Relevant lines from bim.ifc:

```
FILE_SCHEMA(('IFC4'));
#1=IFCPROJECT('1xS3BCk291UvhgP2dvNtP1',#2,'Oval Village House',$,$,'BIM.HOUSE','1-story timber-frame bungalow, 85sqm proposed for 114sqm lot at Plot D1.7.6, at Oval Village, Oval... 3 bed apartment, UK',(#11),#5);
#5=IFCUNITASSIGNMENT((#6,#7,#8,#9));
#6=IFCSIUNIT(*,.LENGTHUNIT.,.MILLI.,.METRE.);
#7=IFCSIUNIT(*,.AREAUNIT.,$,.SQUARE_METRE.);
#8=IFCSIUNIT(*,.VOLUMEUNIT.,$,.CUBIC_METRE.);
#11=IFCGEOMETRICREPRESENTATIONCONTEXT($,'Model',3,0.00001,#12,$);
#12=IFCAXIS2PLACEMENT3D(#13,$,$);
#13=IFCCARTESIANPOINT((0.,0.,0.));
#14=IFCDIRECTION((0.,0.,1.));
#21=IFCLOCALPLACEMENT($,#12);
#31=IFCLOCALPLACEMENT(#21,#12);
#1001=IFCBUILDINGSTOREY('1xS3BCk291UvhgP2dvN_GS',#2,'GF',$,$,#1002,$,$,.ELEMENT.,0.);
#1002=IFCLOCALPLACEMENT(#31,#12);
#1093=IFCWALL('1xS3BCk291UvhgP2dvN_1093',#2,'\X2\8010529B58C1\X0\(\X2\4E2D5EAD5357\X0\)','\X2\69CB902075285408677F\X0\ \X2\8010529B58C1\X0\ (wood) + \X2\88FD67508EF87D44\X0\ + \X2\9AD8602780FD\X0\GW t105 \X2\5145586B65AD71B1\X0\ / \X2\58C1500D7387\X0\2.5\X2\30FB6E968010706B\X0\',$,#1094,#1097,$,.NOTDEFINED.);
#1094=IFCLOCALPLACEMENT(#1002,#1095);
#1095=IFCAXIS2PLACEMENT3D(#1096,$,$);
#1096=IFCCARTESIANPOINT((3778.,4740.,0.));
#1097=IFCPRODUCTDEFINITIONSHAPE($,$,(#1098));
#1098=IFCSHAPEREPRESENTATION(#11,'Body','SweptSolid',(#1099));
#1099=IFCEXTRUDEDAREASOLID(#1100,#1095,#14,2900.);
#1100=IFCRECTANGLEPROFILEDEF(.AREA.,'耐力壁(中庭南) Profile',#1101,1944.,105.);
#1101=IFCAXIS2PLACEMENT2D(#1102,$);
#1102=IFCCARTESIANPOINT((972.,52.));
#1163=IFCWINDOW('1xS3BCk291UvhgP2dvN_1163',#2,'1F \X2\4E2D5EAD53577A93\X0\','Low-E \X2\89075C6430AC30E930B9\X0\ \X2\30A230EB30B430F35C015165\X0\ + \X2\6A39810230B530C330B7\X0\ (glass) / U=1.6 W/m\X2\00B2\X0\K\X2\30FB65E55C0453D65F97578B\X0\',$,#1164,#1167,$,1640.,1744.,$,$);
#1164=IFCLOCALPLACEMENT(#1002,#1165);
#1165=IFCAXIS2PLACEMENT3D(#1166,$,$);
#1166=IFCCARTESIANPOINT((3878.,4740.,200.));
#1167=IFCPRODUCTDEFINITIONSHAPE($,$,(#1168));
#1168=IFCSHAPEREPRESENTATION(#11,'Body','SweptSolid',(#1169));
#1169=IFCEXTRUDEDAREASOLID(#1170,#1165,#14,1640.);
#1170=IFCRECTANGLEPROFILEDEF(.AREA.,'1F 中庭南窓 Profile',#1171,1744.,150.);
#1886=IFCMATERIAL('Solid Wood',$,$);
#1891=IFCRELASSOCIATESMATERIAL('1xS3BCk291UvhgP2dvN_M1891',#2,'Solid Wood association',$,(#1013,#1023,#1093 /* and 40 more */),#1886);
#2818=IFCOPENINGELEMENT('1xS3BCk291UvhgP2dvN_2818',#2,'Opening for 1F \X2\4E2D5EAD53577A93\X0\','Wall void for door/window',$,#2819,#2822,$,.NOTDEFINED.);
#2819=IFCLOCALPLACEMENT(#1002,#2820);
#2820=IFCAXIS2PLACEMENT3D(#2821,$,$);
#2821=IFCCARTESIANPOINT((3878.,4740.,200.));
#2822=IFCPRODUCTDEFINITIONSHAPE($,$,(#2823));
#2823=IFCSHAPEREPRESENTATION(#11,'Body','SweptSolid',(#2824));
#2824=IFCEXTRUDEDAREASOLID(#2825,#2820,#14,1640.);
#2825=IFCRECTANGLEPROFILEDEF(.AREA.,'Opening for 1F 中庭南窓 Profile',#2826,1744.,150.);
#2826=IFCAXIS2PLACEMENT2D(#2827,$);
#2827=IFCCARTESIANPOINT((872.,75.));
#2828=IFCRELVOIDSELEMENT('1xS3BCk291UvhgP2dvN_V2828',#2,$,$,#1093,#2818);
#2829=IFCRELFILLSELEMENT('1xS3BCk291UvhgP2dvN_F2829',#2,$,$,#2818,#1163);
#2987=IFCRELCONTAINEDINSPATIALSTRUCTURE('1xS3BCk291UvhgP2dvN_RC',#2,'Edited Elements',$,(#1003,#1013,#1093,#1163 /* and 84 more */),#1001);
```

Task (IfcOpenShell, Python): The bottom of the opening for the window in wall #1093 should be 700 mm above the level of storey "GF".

```python
import numpy as np
import ifcopenshell
import ifcopenshell.api.geometry
import ifcopenshell.geom
import ifcopenshell.util.element
import ifcopenshell.util.placement
import ifcopenshell.util.shape
import ifcopenshell.util.unit

model = ifcopenshell.open("bim.ifc")
unit_scale = ifcopenshell.util.unit.calculate_unit_scale(model)

window = model.by_guid("1xS3BCk291UvhgP2dvN_1163")
opening = window.FillsVoids[0].RelatingOpeningElement
storey = ifcopenshell.util.element.get_container(window, ifc_class="IfcBuildingStorey")
level = ifcopenshell.util.placement.get_local_placement(storey.ObjectPlacement)[2, 3]

# The opening's origin need not be at the sill, so measure its lowest point.
shape = ifcopenshell.geom.create_shape(ifcopenshell.geom.settings(), opening)
bottom = ifcopenshell.util.shape.get_shape_bottom_elevation(shape, shape.geometry) / unit_scale
dz = level + 0.7 / unit_scale - bottom

shift = np.array([0.0, 0.0, dz])
# The window is not placed relative to its opening, so move both.
for product in (opening, window):
    matrix = ifcopenshell.util.placement.get_local_placement(product.ObjectPlacement)
    matrix[:3, 3] += shift
    ifcopenshell.api.geometry.edit_object_placement(model, product=product, matrix=matrix, is_si=False)

print(f"moved by {dz * unit_scale:+.3f} m")

model.write("bim_rev.ifc")
```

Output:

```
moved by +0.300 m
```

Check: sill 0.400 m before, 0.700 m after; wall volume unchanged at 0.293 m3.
